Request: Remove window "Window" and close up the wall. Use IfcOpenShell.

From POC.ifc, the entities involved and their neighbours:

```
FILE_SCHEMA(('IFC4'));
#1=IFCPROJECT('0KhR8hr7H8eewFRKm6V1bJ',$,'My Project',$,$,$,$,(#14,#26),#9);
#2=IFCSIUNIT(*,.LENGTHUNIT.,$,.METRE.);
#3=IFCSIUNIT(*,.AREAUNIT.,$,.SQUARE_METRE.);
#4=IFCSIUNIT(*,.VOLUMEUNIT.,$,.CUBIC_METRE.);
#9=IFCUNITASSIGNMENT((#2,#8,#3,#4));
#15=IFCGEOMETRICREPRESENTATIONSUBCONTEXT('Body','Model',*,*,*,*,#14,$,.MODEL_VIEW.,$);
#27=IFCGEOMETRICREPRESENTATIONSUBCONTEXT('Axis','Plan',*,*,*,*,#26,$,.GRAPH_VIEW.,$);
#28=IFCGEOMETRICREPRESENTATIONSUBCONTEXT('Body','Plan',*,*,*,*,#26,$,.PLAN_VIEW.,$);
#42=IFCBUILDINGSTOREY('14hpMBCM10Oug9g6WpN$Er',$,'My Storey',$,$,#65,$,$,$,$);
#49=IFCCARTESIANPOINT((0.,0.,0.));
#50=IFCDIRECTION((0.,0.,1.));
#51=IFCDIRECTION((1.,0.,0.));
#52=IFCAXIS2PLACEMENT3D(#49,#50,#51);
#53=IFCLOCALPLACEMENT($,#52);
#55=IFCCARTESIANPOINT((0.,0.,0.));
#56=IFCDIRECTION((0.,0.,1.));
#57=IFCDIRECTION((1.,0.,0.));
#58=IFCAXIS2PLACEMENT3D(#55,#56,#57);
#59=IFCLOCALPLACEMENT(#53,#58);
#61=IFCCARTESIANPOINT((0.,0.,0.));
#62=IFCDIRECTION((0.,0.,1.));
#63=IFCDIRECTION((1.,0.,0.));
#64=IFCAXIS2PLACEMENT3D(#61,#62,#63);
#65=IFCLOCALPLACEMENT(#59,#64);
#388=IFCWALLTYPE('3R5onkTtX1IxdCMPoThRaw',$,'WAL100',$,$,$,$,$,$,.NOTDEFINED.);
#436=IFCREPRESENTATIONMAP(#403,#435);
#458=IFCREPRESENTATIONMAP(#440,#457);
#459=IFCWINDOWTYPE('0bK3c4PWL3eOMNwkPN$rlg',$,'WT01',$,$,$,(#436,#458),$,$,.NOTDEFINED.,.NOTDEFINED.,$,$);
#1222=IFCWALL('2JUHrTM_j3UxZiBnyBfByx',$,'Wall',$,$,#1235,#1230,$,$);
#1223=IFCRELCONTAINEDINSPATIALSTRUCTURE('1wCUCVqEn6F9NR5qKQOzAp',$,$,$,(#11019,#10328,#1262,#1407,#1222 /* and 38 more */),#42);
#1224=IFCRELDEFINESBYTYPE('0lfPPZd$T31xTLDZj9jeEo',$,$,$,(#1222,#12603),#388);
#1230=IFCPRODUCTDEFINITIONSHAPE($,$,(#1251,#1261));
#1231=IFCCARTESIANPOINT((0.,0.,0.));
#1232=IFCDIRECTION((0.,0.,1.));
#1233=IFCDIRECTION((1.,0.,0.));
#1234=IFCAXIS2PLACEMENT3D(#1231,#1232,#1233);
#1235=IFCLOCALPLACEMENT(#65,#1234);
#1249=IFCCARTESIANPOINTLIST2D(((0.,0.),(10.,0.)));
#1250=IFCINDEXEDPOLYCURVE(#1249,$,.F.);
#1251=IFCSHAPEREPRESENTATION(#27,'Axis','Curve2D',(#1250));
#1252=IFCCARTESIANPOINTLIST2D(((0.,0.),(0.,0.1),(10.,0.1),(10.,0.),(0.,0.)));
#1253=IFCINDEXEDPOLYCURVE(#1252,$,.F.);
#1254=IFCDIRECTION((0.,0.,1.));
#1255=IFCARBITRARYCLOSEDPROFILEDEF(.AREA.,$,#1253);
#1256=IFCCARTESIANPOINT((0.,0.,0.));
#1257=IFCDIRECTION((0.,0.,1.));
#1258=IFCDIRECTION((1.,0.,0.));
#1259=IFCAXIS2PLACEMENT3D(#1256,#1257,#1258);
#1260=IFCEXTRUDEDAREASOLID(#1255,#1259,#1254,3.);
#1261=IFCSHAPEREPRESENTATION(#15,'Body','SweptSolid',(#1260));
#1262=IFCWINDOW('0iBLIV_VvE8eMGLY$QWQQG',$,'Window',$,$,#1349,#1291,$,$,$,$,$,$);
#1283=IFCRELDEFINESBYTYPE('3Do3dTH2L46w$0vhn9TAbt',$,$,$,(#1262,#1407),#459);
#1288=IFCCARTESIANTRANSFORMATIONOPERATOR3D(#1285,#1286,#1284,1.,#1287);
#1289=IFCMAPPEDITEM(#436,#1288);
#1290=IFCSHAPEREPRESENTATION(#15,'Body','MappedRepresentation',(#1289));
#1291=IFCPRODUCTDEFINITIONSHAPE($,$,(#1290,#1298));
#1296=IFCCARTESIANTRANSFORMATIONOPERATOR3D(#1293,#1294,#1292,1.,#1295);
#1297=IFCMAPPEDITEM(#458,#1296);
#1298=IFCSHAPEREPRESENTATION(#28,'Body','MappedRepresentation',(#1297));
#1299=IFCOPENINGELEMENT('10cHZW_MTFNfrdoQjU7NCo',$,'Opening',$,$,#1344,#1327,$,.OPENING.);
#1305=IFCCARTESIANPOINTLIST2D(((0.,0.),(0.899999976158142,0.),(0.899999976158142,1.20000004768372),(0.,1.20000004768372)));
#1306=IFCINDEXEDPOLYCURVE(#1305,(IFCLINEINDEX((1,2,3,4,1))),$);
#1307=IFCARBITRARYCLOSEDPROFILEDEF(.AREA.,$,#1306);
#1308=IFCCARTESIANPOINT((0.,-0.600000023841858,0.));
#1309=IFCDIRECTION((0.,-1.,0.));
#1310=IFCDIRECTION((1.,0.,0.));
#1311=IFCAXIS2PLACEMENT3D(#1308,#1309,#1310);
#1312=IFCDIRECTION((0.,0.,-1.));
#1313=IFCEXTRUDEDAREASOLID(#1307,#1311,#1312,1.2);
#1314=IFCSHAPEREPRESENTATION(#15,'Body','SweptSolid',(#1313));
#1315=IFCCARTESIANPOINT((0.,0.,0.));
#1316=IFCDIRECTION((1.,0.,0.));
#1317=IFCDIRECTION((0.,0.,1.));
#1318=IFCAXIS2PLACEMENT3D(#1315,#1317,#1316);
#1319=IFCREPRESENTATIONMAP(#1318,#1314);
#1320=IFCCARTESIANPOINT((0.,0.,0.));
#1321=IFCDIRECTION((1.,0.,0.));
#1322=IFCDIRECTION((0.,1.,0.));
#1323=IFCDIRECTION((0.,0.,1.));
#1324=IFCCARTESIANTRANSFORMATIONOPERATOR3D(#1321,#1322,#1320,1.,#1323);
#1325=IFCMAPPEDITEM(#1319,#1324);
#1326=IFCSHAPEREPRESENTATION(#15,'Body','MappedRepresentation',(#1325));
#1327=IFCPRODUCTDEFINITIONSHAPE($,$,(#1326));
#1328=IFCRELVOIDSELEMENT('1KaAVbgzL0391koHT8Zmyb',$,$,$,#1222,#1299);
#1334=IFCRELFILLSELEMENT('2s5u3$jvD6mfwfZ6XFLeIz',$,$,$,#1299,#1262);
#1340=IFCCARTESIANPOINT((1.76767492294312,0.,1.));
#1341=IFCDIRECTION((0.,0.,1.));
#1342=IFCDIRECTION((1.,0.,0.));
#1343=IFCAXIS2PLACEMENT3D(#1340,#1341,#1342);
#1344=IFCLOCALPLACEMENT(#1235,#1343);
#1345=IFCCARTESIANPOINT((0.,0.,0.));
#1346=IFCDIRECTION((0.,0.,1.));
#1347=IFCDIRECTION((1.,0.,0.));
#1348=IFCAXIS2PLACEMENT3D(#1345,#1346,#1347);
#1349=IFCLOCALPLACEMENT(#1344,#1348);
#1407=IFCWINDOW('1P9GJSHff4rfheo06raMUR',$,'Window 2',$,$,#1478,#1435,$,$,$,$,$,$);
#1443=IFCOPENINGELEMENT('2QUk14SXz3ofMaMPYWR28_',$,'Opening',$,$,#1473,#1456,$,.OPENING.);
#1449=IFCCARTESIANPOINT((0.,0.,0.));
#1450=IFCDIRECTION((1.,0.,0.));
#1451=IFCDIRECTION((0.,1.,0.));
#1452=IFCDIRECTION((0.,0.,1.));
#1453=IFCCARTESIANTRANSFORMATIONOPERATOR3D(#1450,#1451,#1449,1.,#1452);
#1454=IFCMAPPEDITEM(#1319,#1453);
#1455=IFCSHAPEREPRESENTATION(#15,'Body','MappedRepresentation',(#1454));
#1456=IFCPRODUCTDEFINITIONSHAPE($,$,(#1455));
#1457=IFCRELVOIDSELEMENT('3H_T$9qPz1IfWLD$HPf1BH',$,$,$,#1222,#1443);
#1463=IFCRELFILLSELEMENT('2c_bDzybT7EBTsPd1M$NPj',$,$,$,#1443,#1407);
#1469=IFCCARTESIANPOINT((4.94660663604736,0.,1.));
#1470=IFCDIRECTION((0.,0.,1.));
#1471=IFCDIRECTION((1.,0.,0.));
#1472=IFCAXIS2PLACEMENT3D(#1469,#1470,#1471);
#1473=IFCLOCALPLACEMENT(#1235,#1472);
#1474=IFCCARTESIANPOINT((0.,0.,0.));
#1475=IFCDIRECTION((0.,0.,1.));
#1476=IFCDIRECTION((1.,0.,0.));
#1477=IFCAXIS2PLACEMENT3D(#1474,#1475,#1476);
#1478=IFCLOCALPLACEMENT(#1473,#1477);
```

```python
import ifcopenshell
import ifcopenshell.api.feature
import ifcopenshell.api.root
import ifcopenshell.geom
import ifcopenshell.util.shape

model = ifcopenshell.open("POC.ifc")
settings = ifcopenshell.geom.settings()


def volume(element):
    """Net volume in cubic metres, openings subtracted."""
    shape = ifcopenshell.geom.create_shape(settings, element)
    return ifcopenshell.util.shape.get_volume(shape.geometry)


window = model.by_id(1262)
opening = window.FillsVoids[0].RelatingOpeningElement
wall = opening.VoidsElements[0].RelatingBuildingElement
before = volume(wall)

ifcopenshell.api.root.remove_product(model, product=window)
ifcopenshell.api.feature.remove_feature(model, feature=opening)

after = volume(wall)

print(f"wall volume {before:.3f} -> {after:.3f} m3")

model.write("POC-out.ifc")
```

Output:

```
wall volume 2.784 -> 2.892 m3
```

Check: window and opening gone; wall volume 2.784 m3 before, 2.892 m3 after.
